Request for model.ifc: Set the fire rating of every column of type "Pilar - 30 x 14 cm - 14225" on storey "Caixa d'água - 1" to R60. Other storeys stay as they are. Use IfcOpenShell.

First a look at what the model holds.

```python
import ifcopenshell
import ifcopenshell.util.element

model = ifcopenshell.open("model.ifc")
print(model.schema)
storey = next(s for s in model.by_type("IfcBuildingStorey") if s.Name == "Caixa d'água - 1")
columns = [e for e in ifcopenshell.util.element.get_decomposition(storey) if e.is_a("IfcColumn")]
seen = {}
for e in columns:
    element_type = ifcopenshell.util.element.get_type(e)
    key = (element_type.Name if element_type != e and element_type else None, ifcopenshell.util.element.get_pset(e, "Pset_ColumnCommon", "FireRating"))
    seen[key] = seen.get(key, 0) + 1
for (name, value), count in sorted(seen.items(), key=str):
    print(count, "x", name, "|", value)
```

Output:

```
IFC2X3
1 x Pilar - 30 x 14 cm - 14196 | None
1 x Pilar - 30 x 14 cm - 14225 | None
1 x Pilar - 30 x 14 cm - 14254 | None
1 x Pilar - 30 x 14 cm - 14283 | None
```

```python
import ifcopenshell
import ifcopenshell.api.pset
import ifcopenshell.util.element

model = ifcopenshell.open("model.ifc")

storey = next(s for s in model.by_type("IfcBuildingStorey") if s.Name == "Caixa d'água - 1")
columns = [e for e in ifcopenshell.util.element.get_decomposition(storey) if e.is_a("IfcColumn")]

count = 0
for e in columns:
    element_type = ifcopenshell.util.element.get_type(e)
    if element_type in (None, e) or element_type.Name != "Pilar - 30 x 14 cm - 14225":
        continue
    # add_pset returns the element's existing set when there is one.
    pset = ifcopenshell.api.pset.add_pset(model, product=e, name="Pset_ColumnCommon")
    ifcopenshell.api.pset.edit_pset(model, pset=pset, properties={"FireRating": "R60"})
    count += 1

print(count, "columns updated")

model.write("model_rev.ifc")
```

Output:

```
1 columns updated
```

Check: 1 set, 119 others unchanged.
